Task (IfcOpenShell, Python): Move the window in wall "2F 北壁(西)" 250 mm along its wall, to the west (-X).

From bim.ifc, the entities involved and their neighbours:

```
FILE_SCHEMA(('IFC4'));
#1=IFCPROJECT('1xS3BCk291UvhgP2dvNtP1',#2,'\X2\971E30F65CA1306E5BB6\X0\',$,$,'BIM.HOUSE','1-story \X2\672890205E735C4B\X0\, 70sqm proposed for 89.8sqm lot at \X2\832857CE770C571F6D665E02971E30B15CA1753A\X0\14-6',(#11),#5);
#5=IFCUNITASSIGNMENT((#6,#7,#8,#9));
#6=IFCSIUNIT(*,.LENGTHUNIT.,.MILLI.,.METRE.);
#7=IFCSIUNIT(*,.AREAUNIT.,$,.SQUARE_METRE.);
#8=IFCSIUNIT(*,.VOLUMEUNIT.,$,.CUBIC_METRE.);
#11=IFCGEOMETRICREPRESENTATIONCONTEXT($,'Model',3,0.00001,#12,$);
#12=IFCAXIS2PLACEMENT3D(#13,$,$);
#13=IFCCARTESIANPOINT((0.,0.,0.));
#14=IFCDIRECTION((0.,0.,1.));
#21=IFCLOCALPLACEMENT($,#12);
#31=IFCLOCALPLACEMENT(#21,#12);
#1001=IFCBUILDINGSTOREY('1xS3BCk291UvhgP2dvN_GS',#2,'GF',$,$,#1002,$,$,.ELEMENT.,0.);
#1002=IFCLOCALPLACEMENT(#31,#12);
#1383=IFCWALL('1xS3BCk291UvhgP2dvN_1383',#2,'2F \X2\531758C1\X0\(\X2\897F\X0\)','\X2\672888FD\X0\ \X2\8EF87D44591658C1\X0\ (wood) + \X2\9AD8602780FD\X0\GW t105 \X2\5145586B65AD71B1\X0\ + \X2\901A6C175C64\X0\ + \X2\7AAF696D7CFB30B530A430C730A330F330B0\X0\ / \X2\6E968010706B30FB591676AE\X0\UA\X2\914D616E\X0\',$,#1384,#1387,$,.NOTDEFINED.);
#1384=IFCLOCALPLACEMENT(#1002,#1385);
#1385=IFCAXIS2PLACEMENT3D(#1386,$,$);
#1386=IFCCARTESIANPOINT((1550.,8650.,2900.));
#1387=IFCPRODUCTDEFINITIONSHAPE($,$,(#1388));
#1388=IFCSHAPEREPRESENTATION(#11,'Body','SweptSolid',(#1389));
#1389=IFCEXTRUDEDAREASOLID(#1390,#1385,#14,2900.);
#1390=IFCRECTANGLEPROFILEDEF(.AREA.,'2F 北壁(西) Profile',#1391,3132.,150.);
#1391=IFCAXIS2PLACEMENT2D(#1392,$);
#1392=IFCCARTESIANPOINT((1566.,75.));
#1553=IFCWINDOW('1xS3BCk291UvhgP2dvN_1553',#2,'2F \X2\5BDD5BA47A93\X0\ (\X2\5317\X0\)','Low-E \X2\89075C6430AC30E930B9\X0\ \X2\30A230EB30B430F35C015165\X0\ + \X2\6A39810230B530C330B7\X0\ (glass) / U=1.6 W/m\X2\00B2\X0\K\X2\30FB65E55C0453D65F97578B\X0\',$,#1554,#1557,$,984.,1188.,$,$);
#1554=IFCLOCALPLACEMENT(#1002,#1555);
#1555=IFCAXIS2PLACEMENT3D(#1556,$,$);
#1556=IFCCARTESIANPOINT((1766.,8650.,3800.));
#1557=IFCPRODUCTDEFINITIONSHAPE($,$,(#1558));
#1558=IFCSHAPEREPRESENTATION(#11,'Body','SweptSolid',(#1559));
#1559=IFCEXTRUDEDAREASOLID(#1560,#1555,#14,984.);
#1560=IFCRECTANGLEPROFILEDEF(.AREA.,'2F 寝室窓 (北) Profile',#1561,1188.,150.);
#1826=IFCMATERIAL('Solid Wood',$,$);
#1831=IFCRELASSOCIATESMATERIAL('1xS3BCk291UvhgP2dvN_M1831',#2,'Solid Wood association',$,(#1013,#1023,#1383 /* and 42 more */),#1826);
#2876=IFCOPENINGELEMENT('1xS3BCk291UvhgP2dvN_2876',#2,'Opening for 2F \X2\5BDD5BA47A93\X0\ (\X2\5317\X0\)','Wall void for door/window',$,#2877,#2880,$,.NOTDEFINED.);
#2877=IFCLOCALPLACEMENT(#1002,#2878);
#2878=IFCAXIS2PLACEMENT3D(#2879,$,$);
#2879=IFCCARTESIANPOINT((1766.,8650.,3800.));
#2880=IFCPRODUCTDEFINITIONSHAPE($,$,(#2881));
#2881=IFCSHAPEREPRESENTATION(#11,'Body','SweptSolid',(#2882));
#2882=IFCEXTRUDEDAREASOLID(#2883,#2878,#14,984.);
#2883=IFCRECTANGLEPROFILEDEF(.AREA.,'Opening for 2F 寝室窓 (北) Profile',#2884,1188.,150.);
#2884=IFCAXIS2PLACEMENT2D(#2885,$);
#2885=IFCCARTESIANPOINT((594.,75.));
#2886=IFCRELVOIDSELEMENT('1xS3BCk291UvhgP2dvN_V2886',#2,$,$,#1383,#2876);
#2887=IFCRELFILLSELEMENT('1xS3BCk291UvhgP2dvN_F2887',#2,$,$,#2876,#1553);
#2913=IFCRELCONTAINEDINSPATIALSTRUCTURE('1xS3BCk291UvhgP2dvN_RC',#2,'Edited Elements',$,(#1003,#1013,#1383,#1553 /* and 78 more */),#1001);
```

```python
import ifcopenshell
import ifcopenshell.api.geometry
import ifcopenshell.util.placement
import ifcopenshell.util.unit

model = ifcopenshell.open("bim.ifc")
unit_scale = ifcopenshell.util.unit.calculate_unit_scale(model)

window = model.by_guid("1xS3BCk291UvhgP2dvN_1553")
opening = window.FillsVoids[0].RelatingOpeningElement
wall = opening.VoidsElements[0].RelatingBuildingElement

wall_matrix = ifcopenshell.util.placement.get_local_placement(wall.ObjectPlacement)
shift = wall_matrix[:3, 0] * -0.25 / unit_scale
before = ifcopenshell.util.placement.get_local_placement(window.ObjectPlacement)[:3, 3].copy()

# The window is not placed relative to its opening, so move both.
for product in (opening, window):
    matrix = ifcopenshell.util.placement.get_local_placement(product.ObjectPlacement)
    matrix[:3, 3] += shift
    ifcopenshell.api.geometry.edit_object_placement(model, product=product, matrix=matrix, is_si=False)

after = ifcopenshell.util.placement.get_local_placement(window.ObjectPlacement)[:3, 3]
print("window moved by", (after - before).round(3) + 0.0)

model.write("bim-out.ifc")
```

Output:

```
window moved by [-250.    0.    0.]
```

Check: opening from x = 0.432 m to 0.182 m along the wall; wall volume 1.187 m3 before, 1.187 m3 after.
